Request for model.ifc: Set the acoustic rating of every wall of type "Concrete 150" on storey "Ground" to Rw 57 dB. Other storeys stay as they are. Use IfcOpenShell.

First a look at what the model holds.

```python
import ifcopenshell
import ifcopenshell.util.element

model = ifcopenshell.open("model.ifc")
print(model.schema)
storey = next(s for s in model.by_type("IfcBuildingStorey") if s.Name == "Ground")
walls = [e for e in ifcopenshell.util.element.get_decomposition(storey) if e.is_a("IfcWall")]
seen = {}
for e in walls:
    element_type = ifcopenshell.util.element.get_type(e)
    key = (element_type.Name if element_type != e and element_type else None, ifcopenshell.util.element.get_pset(e, "Pset_WallCommon", "AcousticRating"))
    seen[key] = seen.get(key, 0) + 1
for (name, value), count in sorted(seen.items(), key=str):
    print(count, "x", name, "|", value)
```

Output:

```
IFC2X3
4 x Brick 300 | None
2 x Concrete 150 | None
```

```python
import ifcopenshell
import ifcopenshell.api.pset
import ifcopenshell.util.element

model = ifcopenshell.open("model.ifc")

storey = next(s for s in model.by_type("IfcBuildingStorey") if s.Name == "Ground")
walls = [e for e in ifcopenshell.util.element.get_decomposition(storey) if e.is_a("IfcWall")]

count = 0
for e in walls:
    element_type = ifcopenshell.util.element.get_type(e)
    if element_type in (None, e) or element_type.Name != "Concrete 150":
        continue
    # add_pset returns the element's existing set when there is one.
    pset = ifcopenshell.api.pset.add_pset(model, product=e, name="Pset_WallCommon")
    ifcopenshell.api.pset.edit_pset(model, pset=pset, properties={"AcousticRating": "Rw 57 dB"})
    count += 1

print(count, "walls updated")

model.write("model_v2.ifc")
```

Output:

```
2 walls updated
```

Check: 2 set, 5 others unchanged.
